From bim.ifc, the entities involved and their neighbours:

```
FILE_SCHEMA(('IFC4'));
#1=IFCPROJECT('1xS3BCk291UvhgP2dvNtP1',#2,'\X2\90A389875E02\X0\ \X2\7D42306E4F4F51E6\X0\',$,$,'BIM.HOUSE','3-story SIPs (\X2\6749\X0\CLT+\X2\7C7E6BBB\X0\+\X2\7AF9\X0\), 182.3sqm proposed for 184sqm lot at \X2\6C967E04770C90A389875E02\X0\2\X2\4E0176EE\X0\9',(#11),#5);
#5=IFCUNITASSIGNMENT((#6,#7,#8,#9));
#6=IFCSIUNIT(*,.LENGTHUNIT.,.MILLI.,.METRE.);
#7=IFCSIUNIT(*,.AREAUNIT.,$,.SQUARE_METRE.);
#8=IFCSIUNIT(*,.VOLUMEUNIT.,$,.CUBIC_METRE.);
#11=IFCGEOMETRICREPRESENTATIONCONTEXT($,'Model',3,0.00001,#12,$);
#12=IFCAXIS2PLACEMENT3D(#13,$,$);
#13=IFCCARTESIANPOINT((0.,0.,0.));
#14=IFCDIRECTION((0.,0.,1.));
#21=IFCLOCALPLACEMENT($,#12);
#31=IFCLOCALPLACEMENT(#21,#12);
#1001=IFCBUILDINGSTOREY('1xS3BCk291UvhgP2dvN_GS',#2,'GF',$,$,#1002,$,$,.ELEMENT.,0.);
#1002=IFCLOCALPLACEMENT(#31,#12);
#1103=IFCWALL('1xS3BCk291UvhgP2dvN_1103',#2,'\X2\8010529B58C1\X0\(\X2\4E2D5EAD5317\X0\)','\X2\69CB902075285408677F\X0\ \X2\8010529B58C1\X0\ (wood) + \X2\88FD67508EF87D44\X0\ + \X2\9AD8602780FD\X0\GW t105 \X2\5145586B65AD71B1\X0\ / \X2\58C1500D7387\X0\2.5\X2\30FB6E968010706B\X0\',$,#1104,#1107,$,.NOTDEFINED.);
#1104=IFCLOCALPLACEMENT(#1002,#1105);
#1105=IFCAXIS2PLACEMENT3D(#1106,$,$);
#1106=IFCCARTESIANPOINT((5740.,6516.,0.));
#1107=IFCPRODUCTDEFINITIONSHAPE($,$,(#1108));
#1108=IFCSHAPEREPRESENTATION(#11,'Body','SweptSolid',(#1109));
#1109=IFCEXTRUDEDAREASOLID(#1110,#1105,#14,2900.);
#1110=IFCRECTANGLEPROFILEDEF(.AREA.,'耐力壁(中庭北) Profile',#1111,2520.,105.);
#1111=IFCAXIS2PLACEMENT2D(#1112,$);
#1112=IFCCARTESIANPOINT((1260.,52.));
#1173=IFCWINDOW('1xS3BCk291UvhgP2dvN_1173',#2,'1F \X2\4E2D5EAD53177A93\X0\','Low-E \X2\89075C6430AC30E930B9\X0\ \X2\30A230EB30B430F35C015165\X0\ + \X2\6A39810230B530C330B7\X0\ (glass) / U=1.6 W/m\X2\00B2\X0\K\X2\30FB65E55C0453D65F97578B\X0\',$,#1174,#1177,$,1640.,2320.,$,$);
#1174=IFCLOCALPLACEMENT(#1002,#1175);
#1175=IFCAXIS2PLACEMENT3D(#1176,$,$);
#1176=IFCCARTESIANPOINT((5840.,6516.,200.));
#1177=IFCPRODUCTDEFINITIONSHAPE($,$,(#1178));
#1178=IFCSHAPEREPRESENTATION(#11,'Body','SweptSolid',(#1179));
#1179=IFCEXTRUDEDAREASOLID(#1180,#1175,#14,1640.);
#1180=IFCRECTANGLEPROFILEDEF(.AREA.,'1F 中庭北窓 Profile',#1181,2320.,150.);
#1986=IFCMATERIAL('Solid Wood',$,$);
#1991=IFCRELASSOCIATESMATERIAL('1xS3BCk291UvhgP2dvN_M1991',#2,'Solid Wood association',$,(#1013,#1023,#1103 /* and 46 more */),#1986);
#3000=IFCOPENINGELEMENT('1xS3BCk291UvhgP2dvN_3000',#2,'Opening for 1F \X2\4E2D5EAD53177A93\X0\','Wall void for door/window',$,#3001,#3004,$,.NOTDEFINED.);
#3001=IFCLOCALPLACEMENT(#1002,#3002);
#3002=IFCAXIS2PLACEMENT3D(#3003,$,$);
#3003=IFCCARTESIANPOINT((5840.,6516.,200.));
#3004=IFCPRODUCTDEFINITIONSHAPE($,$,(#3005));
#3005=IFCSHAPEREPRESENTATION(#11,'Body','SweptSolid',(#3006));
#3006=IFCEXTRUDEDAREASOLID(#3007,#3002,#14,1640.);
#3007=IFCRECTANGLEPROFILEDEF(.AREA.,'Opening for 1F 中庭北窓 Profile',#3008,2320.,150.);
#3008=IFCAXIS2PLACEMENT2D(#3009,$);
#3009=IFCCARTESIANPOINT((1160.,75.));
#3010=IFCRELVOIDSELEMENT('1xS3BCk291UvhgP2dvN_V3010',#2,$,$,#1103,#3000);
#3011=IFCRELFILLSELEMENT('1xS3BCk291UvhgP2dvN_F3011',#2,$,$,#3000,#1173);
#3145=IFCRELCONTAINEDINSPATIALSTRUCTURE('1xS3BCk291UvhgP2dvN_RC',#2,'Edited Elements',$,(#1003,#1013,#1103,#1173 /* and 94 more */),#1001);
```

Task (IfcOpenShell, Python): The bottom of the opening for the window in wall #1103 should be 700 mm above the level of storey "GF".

```python
import numpy as np
import ifcopenshell
import ifcopenshell.api.geometry
import ifcopenshell.geom
import ifcopenshell.util.element
import ifcopenshell.util.placement
import ifcopenshell.util.shape
import ifcopenshell.util.unit

model = ifcopenshell.open("bim.ifc")
unit_scale = ifcopenshell.util.unit.calculate_unit_scale(model)

window = model.by_id(1173)
opening = window.FillsVoids[0].RelatingOpeningElement
storey = ifcopenshell.util.element.get_container(window, ifc_class="IfcBuildingStorey")
level = ifcopenshell.util.placement.get_local_placement(storey.ObjectPlacement)[2, 3]

# The opening's origin need not be at the sill, so measure its lowest point.
shape = ifcopenshell.geom.create_shape(ifcopenshell.geom.settings(), opening)
bottom = ifcopenshell.util.shape.get_shape_bottom_elevation(shape, shape.geometry) / unit_scale
dz = level + 700.0 - bottom

shift = np.array([0.0, 0.0, dz])
# The window is not placed relative to its opening, so move both.
for product in (opening, window):
    matrix = ifcopenshell.util.placement.get_local_placement(product.ObjectPlacement)
    matrix[:3, 3] += shift
    ifcopenshell.api.geometry.edit_object_placement(model, product=product, matrix=matrix, is_si=False)

print(f"moved by {dz * unit_scale:+.3f} m")

model.write("bim-out.ifc")
```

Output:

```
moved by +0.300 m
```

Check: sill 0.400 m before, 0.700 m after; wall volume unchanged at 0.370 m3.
